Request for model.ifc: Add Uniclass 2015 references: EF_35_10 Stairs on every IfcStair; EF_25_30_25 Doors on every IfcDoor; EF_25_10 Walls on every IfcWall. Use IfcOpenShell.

First a look at what the model holds.

```python
import ifcopenshell

model = ifcopenshell.open("model.ifc")
print(model.schema)
print("classifications:", [c.Name for c in model.by_type("IfcClassification")])
for ifc_class in ("IfcDoor", "IfcRoof", "IfcStair", "IfcWall", "IfcWindow"):
    print(ifc_class, len(model.by_type(ifc_class)))
```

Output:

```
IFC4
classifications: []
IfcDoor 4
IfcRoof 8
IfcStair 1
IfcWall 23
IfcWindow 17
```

```python
import ifcopenshell
import ifcopenshell.api.classification

model = ifcopenshell.open("model.ifc")

system = ifcopenshell.api.classification.add_classification(model, classification="Uniclass 2015")

codes = {
    "IfcStair": ("EF_35_10", "Stairs"),
    "IfcDoor": ("EF_25_30_25", "Doors"),
    "IfcWall": ("EF_25_10", "Walls"),
}
for ifc_class, (code, name) in codes.items():
    products = model.by_type(ifc_class)
    ifcopenshell.api.classification.add_reference(
        model, products=products, classification=system, identification=code, name=name
    )
    print(code, len(products))

model.write("model_v2.ifc")
```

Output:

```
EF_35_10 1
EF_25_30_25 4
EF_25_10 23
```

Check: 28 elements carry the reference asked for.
